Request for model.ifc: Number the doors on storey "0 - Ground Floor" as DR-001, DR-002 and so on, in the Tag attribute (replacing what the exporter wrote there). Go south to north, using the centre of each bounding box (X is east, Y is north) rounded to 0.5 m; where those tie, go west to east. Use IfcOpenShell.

First a look at what the model holds.

```python
import ifcopenshell
import ifcopenshell.util.element
import ifcopenshell.util.placement

model = ifcopenshell.open("model.ifc")
print(model.schema)
storey = next(s for s in model.by_type("IfcBuildingStorey") if s.Name == "0 - Ground Floor")
doors = [e for e in ifcopenshell.util.element.get_decomposition(storey) if e.is_a("IfcDoor")]
for e in sorted(doors, key=lambda e: e.id()):
    origin = ifcopenshell.util.placement.get_local_placement(e.ObjectPlacement)[:3, 3]
    print(e.id(), e.Tag, e.Name, origin.round(2) + 0.0, sep=" | ")
```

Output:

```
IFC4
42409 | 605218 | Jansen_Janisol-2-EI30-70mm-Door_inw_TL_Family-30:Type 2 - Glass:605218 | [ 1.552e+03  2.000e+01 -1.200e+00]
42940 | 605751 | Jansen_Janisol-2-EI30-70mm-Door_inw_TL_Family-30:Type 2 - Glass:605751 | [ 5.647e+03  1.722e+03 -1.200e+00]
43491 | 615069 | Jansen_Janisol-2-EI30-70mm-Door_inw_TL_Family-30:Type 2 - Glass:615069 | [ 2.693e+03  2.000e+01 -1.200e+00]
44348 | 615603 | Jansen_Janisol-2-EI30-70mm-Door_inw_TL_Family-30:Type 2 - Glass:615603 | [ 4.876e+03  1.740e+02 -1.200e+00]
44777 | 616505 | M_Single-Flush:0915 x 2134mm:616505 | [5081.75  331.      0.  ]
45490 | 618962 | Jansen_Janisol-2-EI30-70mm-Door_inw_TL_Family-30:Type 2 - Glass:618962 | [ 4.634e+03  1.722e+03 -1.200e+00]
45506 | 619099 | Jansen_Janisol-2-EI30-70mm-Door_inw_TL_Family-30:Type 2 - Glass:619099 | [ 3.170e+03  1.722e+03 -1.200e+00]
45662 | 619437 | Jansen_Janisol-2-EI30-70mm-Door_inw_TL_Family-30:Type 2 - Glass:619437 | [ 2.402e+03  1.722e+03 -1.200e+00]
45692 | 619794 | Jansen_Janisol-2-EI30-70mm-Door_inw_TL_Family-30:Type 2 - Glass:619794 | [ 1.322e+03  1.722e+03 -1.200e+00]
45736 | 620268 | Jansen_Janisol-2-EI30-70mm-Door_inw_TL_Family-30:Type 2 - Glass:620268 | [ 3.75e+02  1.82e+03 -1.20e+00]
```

```python
import ifcopenshell
import ifcopenshell.geom
import ifcopenshell.util.element
import ifcopenshell.util.shape

model = ifcopenshell.open("model.ifc")
settings = ifcopenshell.geom.settings()
settings.set("use-world-coords", True)


def centre(element):
    shape = ifcopenshell.geom.create_shape(settings, element)
    return ifcopenshell.util.shape.get_bbox_centroid(shape.geometry)


storey = next(s for s in model.by_type("IfcBuildingStorey") if s.Name == "0 - Ground Floor")
doors = [e for e in ifcopenshell.util.element.get_decomposition(storey) if e.is_a("IfcDoor")]

# Insertion points can sit at a corner or the storey origin, so sort by the geometry (in metres).
centres = {e: centre(e) for e in doors}
doors.sort(key=lambda e: (round(centres[e][1] / 0.5), centres[e][0]))

for i, e in enumerate(doors, start=1):
    number = f"DR-0{i:02d}"
    e.Tag = number
    print(e.id(), number)

model.write("model_edited.ifc")
```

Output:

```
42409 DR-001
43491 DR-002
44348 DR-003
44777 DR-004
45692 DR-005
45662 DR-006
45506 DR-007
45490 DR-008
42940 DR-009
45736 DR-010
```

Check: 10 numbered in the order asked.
